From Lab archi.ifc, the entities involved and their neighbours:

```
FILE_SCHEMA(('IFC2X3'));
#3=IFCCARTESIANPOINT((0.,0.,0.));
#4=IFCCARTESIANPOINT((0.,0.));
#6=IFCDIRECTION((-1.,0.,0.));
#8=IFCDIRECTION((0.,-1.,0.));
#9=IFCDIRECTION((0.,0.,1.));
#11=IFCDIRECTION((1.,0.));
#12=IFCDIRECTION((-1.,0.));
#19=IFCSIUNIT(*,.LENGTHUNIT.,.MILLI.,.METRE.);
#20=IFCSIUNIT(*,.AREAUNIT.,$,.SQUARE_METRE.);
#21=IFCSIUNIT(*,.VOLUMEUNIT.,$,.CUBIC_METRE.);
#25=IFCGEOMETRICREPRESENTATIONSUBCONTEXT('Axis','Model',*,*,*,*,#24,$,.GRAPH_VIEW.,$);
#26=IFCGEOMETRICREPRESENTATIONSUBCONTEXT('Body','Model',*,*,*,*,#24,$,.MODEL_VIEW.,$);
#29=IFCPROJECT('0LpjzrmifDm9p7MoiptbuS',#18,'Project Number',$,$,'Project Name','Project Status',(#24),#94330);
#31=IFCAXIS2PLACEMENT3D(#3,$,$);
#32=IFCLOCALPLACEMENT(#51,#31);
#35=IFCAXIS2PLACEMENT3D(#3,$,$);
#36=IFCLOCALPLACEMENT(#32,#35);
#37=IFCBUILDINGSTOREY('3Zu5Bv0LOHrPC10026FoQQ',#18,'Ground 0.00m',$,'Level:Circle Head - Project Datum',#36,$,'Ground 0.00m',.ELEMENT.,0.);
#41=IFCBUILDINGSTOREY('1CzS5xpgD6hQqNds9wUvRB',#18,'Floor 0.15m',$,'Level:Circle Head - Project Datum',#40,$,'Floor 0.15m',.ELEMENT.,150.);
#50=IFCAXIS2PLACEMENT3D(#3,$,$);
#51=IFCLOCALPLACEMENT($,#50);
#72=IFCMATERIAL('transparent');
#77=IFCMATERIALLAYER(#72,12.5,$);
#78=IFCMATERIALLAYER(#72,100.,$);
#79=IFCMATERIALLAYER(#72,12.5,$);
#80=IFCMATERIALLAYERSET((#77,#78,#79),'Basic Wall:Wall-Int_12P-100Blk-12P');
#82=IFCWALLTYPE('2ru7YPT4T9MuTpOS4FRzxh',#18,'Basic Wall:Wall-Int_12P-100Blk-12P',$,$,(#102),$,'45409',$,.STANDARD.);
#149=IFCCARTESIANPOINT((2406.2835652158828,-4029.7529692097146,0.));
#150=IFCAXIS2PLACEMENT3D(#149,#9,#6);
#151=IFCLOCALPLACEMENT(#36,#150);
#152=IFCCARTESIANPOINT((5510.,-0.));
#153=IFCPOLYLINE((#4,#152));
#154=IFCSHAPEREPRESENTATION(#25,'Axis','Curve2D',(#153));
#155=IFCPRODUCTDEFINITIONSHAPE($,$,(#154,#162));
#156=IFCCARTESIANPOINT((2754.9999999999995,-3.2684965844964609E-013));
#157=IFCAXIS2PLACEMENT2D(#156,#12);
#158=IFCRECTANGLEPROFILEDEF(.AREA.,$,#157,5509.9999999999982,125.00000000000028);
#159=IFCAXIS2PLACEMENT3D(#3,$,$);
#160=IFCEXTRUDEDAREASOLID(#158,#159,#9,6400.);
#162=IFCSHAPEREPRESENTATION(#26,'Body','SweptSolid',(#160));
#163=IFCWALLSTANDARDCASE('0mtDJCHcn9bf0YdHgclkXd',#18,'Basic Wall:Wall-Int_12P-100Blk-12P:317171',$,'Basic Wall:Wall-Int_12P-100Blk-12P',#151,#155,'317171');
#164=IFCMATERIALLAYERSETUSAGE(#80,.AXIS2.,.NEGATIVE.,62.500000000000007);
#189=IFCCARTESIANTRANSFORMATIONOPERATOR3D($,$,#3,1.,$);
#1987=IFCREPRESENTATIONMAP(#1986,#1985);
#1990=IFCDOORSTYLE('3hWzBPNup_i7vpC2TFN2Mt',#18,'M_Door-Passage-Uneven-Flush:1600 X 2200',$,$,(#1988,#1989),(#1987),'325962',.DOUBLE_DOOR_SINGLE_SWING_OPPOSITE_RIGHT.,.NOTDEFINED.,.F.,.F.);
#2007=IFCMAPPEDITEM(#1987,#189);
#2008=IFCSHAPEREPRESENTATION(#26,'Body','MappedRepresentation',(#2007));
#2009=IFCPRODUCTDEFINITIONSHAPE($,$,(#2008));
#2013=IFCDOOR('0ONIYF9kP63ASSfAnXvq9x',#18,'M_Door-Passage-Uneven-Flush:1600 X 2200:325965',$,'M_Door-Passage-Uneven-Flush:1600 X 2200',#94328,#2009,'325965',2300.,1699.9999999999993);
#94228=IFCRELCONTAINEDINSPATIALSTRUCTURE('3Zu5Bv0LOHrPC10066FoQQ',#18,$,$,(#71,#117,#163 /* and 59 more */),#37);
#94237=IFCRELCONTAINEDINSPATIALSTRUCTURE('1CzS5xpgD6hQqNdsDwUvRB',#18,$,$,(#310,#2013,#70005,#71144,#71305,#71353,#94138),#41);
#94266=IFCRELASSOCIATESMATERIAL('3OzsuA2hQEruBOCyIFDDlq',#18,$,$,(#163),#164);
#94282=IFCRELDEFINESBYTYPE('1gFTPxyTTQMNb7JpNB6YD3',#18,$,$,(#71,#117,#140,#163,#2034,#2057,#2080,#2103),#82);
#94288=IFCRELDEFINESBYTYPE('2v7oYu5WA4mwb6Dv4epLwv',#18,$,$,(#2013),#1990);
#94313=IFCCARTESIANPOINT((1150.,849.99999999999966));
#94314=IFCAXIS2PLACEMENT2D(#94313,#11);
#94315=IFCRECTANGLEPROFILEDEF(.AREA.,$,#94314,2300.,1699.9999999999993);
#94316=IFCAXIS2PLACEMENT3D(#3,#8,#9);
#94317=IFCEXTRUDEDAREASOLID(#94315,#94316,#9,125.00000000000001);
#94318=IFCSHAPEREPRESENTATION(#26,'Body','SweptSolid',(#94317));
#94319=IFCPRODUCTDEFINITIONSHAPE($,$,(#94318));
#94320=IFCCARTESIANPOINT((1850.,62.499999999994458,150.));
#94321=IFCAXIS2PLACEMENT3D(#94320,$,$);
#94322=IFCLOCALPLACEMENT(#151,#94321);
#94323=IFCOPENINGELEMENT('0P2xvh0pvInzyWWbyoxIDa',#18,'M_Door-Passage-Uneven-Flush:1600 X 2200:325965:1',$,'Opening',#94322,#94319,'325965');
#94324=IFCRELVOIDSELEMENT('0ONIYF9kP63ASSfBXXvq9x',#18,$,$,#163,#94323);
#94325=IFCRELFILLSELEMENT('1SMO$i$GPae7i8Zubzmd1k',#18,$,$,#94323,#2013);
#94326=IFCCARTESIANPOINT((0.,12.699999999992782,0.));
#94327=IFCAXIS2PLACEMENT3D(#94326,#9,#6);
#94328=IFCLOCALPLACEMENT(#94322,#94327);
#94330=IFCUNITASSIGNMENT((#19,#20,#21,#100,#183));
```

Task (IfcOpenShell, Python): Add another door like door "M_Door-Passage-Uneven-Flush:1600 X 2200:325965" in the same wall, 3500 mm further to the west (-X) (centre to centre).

```python
import ifcopenshell
import ifcopenshell.api.feature
import ifcopenshell.api.geometry
import ifcopenshell.api.root
import ifcopenshell.geom
import ifcopenshell.util.element
import ifcopenshell.util.placement
import ifcopenshell.util.shape

model = ifcopenshell.open("Lab archi.ifc")
settings = ifcopenshell.geom.settings()


def volume(element):
    """Net volume in cubic metres, openings subtracted."""
    shape = ifcopenshell.geom.create_shape(settings, element)
    return ifcopenshell.util.shape.get_volume(shape.geometry)


def reuse_history(source, copy):
    """copy_class also copies each property set's owner history, people and application; keep the originals."""
    for rel in copy.IsDefinedBy:
        if rel.is_a("IfcRelDefinesByProperties") and (history := rel.RelatingPropertyDefinition.OwnerHistory):
            rel.RelatingPropertyDefinition.OwnerHistory = source.OwnerHistory
            ifcopenshell.util.element.remove_deep2(model, history)


door = model.by_guid("0ONIYF9kP63ASSfAnXvq9x")
opening = door.FillsVoids[0].RelatingOpeningElement
wall = opening.VoidsElements[0].RelatingBuildingElement
before = volume(wall)
shift = ifcopenshell.util.placement.get_local_placement(wall.ObjectPlacement)[:3, 0] * 3500.0

# copy_class copies the void relationship, type, container and properties, but no geometry.
new_opening = ifcopenshell.api.root.copy_class(model, product=opening)
new_opening.Representation = ifcopenshell.util.element.copy_deep(
    model, opening.Representation, exclude=["IfcGeometricRepresentationContext", "IfcRepresentationMap"]
)
new_opening.Name = "M_Door-Passage-Uneven-Flush:1600 X 2200"
new_opening.Tag = None
new_door = ifcopenshell.api.root.copy_class(model, product=door)
new_door.Representation = ifcopenshell.util.element.copy_deep(
    model, door.Representation, exclude=["IfcGeometricRepresentationContext", "IfcRepresentationMap"]
)
new_door.Name = "M_Door-Passage-Uneven-Flush:1600 X 2200"
new_door.Tag = None
reuse_history(door, new_door)
fills = ifcopenshell.api.feature.add_filling(model, opening=new_opening, element=new_door)
fills.OwnerHistory = new_door.OwnerHistory  # required in IFC2X3

for old, new in ((opening, new_opening), (door, new_door)):
    matrix = ifcopenshell.util.placement.get_local_placement(old.ObjectPlacement)
    matrix[:3, 3] += shift
    ifcopenshell.api.geometry.edit_object_placement(model, product=new, matrix=matrix, is_si=False)

after = volume(wall)

print(f"wall volume {before:.3f} -> {after:.3f} m3")

model.write("Lab archi_updated.ifc")
```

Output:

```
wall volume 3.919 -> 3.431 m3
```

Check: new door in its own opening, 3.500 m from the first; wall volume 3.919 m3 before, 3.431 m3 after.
